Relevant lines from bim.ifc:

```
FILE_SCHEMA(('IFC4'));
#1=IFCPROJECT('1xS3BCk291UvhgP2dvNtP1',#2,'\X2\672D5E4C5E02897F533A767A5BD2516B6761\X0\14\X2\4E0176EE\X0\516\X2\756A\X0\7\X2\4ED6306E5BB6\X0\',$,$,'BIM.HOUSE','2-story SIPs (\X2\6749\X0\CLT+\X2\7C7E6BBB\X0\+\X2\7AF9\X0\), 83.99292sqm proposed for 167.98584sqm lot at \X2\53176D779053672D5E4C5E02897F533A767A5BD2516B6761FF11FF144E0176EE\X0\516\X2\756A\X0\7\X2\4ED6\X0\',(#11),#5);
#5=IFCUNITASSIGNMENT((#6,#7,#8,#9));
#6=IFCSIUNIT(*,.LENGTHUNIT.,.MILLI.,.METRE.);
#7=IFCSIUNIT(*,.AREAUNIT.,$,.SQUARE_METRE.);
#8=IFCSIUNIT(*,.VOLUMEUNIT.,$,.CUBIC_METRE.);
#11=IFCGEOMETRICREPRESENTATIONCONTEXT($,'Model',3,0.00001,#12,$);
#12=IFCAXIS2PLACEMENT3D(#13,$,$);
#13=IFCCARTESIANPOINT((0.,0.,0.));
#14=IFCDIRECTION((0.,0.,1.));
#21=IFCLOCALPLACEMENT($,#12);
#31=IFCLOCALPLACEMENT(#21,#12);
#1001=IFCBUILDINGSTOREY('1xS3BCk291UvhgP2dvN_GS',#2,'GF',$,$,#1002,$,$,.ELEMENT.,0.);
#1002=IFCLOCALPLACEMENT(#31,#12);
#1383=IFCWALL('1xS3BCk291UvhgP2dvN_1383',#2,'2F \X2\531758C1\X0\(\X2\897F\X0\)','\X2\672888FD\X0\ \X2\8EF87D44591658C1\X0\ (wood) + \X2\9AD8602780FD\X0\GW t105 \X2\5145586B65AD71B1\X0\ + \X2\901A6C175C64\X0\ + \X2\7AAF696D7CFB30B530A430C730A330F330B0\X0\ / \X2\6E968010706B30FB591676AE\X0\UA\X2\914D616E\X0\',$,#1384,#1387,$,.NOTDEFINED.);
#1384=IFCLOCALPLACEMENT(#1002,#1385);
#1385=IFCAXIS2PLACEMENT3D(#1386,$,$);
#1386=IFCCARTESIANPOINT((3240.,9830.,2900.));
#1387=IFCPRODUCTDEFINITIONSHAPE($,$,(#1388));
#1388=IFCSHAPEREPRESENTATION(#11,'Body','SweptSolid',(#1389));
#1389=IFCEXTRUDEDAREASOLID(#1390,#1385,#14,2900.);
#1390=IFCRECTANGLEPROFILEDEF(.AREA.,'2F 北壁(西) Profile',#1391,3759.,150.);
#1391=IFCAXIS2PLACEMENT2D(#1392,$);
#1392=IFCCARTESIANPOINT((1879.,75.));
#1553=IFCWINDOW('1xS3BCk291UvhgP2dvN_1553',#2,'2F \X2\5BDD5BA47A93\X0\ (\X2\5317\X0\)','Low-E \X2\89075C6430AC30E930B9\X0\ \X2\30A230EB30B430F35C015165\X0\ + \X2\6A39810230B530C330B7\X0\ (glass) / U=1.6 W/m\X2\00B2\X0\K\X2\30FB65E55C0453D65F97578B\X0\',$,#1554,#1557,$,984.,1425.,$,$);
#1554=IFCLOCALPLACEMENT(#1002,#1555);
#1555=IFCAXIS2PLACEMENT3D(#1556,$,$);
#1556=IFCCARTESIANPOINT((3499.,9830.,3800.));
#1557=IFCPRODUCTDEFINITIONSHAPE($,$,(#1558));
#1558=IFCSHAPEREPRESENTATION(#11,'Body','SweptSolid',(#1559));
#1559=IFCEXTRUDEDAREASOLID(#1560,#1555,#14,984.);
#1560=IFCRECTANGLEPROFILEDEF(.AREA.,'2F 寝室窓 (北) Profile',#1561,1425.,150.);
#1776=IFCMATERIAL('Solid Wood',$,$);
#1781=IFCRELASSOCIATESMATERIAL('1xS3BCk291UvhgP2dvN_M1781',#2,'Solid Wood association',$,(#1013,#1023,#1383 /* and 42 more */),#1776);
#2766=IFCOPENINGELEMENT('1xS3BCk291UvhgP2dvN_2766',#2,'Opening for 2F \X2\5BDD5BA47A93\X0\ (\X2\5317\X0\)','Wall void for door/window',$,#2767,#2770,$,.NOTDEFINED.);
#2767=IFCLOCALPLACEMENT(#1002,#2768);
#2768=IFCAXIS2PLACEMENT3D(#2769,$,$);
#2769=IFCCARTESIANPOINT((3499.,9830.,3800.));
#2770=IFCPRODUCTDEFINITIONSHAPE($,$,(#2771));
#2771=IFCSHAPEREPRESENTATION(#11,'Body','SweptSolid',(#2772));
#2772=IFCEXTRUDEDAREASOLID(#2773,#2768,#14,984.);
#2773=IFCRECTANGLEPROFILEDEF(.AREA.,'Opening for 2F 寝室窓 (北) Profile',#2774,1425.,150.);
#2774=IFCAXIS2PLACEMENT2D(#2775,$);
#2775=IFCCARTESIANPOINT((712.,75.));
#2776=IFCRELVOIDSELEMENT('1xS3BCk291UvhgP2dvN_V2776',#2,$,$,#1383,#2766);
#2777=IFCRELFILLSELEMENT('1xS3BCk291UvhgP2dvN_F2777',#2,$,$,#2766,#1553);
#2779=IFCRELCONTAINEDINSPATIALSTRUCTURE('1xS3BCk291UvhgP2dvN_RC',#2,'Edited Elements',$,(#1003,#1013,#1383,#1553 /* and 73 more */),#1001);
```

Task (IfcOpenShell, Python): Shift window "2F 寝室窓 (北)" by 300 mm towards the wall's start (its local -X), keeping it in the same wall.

```python
import ifcopenshell
import ifcopenshell.api.geometry
import ifcopenshell.util.placement
import ifcopenshell.util.unit

model = ifcopenshell.open("bim.ifc")
unit_scale = ifcopenshell.util.unit.calculate_unit_scale(model)

window = model.by_guid("1xS3BCk291UvhgP2dvN_1553")
opening = window.FillsVoids[0].RelatingOpeningElement
wall = opening.VoidsElements[0].RelatingBuildingElement

wall_matrix = ifcopenshell.util.placement.get_local_placement(wall.ObjectPlacement)
shift = wall_matrix[:3, 0] * -0.3 / unit_scale
before = ifcopenshell.util.placement.get_local_placement(window.ObjectPlacement)[:3, 3].copy()

# The window is not placed relative to its opening, so move both.
for product in (opening, window):
    matrix = ifcopenshell.util.placement.get_local_placement(product.ObjectPlacement)
    matrix[:3, 3] += shift
    ifcopenshell.api.geometry.edit_object_placement(model, product=product, matrix=matrix, is_si=False)

after = ifcopenshell.util.placement.get_local_placement(window.ObjectPlacement)[:3, 3]
print("window moved by", (after - before).round(3) + 0.0)

model.write("bim-out.ifc")
```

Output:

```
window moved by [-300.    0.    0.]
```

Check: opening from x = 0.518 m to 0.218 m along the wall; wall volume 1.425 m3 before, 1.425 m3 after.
